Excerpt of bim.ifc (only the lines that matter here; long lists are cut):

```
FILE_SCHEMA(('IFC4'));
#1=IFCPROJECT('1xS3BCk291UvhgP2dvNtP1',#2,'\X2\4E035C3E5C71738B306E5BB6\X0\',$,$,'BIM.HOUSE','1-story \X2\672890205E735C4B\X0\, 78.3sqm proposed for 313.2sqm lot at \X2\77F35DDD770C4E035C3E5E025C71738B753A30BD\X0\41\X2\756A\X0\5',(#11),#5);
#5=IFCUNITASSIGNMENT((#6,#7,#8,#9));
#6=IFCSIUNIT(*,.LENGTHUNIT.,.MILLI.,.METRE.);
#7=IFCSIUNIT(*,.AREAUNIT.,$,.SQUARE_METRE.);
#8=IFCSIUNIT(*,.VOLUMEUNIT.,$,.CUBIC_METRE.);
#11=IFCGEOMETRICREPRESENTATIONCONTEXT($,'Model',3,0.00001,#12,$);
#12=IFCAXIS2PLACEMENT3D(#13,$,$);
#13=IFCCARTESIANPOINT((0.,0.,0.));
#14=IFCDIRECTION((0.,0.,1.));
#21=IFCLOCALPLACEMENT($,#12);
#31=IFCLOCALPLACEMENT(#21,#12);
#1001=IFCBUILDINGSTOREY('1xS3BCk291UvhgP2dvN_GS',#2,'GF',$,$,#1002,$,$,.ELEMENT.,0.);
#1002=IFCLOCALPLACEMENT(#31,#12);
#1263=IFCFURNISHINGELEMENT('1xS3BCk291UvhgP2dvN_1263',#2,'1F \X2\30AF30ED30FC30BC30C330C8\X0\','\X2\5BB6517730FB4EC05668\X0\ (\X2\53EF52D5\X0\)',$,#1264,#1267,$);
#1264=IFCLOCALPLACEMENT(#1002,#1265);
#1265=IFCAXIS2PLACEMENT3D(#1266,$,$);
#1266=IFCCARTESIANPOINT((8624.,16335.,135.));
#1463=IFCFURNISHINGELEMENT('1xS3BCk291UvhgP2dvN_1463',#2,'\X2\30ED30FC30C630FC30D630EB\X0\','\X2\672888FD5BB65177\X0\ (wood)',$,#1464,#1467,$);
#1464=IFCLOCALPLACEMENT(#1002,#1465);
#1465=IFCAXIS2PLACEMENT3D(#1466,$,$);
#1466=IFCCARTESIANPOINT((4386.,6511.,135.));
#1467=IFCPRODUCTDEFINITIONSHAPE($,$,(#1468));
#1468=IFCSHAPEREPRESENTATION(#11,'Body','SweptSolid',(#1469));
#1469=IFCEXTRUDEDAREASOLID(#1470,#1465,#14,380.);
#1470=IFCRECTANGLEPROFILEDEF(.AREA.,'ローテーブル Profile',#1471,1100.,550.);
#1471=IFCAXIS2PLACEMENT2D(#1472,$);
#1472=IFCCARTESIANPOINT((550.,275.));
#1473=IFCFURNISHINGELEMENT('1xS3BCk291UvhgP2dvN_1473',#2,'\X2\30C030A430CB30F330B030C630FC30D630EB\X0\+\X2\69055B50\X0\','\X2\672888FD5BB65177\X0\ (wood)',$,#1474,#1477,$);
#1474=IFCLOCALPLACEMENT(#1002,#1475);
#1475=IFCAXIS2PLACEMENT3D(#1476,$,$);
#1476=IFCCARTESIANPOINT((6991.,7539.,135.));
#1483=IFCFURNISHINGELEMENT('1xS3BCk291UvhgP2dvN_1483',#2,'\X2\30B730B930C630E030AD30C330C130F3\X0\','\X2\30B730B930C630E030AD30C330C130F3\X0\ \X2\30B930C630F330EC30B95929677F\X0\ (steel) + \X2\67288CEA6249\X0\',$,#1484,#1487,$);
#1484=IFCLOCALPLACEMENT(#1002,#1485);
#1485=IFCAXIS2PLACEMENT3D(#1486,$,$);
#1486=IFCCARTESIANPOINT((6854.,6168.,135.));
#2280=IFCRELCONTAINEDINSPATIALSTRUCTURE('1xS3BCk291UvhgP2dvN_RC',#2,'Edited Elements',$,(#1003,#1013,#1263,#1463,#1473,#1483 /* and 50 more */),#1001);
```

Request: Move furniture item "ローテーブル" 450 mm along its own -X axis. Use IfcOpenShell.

```python
import ifcopenshell
import ifcopenshell.api.geometry
import ifcopenshell.util.placement
import ifcopenshell.util.unit

model = ifcopenshell.open("bim.ifc")
unit_scale = ifcopenshell.util.unit.calculate_unit_scale(model)

item = model.by_guid("1xS3BCk291UvhgP2dvN_1463")
matrix = ifcopenshell.util.placement.get_local_placement(item.ObjectPlacement)
matrix[:3, 3] -= matrix[:3, 0] * 0.45 / unit_scale
ifcopenshell.api.geometry.edit_object_placement(model, product=item, matrix=matrix, is_si=False)

print(ifcopenshell.util.placement.get_local_placement(item.ObjectPlacement).round(3) + 0.0)

model.write("bim_rev.ifc")
```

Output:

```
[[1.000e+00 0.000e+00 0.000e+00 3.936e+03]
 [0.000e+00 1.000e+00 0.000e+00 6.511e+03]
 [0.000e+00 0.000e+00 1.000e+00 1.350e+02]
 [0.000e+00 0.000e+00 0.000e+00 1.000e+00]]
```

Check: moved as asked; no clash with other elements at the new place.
